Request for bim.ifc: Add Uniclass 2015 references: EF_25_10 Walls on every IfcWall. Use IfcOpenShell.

First a look at what the model holds.

```python
import ifcopenshell

model = ifcopenshell.open("bim.ifc")
print(model.schema)
print("classifications:", [c.Name for c in model.by_type("IfcClassification")])
for ifc_class in ("IfcDoor", "IfcRoof", "IfcStair", "IfcWall", "IfcWindow"):
    print(ifc_class, len(model.by_type(ifc_class)))
```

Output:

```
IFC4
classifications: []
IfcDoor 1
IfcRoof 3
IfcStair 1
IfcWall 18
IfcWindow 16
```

```python
import ifcopenshell
import ifcopenshell.api.classification

model = ifcopenshell.open("bim.ifc")

system = ifcopenshell.api.classification.add_classification(model, classification="Uniclass 2015")

codes = {
    "IfcWall": ("EF_25_10", "Walls"),
}
for ifc_class, (code, name) in codes.items():
    products = model.by_type(ifc_class)
    ifcopenshell.api.classification.add_reference(
        model, products=products, classification=system, identification=code, name=name
    )
    print(code, len(products))

model.write("bim-out.ifc")
```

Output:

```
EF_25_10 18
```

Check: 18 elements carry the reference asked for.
